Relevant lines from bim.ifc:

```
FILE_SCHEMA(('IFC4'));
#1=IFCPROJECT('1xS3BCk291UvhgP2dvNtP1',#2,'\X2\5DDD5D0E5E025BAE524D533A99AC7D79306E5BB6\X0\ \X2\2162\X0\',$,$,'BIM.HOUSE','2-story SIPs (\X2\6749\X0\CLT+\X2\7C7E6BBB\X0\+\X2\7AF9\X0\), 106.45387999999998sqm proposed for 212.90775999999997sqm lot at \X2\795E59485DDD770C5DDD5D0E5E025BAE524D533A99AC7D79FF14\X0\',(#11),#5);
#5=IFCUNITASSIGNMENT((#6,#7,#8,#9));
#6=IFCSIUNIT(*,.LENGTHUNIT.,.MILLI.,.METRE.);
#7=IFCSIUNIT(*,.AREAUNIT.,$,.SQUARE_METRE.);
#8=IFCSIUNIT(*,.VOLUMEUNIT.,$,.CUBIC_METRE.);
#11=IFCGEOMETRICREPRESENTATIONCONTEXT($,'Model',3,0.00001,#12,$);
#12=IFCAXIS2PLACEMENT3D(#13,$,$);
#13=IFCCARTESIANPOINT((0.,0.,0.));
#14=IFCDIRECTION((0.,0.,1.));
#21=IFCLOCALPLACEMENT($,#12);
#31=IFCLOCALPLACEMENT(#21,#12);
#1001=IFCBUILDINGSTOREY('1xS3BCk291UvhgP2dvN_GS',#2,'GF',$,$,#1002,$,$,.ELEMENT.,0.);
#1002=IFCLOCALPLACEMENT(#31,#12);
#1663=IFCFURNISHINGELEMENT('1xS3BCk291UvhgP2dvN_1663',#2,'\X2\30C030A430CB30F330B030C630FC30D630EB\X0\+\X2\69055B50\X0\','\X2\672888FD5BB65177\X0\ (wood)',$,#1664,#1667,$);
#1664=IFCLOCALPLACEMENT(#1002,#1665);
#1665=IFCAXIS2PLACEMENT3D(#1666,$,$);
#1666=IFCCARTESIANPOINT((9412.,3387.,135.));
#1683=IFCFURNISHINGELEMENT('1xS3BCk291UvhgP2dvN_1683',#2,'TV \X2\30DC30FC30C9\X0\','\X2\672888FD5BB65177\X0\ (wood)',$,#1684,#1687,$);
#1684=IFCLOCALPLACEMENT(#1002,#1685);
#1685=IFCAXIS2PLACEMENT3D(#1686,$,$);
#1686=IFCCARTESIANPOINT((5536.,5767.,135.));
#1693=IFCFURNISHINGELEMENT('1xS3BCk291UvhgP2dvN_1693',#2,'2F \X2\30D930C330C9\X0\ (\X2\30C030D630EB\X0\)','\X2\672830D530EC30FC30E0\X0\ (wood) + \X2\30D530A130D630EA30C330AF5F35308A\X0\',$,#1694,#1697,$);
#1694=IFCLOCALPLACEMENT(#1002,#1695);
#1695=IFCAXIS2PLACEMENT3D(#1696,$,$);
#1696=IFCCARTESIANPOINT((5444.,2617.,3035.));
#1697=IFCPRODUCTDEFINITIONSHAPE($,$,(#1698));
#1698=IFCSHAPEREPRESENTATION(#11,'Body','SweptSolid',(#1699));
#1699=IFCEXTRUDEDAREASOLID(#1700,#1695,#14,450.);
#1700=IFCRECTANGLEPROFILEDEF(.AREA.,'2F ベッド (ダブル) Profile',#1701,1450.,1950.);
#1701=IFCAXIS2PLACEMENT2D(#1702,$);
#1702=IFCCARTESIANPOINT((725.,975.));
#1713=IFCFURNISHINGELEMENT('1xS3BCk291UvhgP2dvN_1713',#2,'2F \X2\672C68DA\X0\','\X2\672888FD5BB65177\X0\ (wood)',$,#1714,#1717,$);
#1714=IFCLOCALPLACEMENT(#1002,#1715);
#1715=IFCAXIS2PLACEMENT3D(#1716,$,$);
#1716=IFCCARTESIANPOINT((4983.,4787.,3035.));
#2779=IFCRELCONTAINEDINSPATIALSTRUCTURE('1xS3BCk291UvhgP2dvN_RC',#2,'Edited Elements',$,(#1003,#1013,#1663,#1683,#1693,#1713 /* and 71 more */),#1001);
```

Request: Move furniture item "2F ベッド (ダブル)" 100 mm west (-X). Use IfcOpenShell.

```python
import ifcopenshell
import ifcopenshell.api.geometry
import ifcopenshell.util.placement

model = ifcopenshell.open("bim.ifc")

item = model.by_guid("1xS3BCk291UvhgP2dvN_1693")
matrix = ifcopenshell.util.placement.get_local_placement(item.ObjectPlacement)
matrix[0, 3] -= 100.0
ifcopenshell.api.geometry.edit_object_placement(model, product=item, matrix=matrix, is_si=False)

print(ifcopenshell.util.placement.get_local_placement(item.ObjectPlacement).round(3) + 0.0)

model.write("bim_v2.ifc")
```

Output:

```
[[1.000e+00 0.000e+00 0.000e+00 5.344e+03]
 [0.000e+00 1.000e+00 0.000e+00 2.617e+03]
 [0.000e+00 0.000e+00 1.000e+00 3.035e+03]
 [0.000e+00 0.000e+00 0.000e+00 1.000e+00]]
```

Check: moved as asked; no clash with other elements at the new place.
